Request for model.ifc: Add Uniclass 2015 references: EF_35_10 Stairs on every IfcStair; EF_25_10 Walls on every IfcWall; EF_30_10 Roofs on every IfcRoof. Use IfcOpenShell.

First a look at what the model holds.

```python
import ifcopenshell

model = ifcopenshell.open("model.ifc")
print(model.schema)
print("classifications:", [c.Name for c in model.by_type("IfcClassification")])
for ifc_class in ("IfcDoor", "IfcRoof", "IfcStair", "IfcWall", "IfcWindow"):
    print(ifc_class, len(model.by_type(ifc_class)))
```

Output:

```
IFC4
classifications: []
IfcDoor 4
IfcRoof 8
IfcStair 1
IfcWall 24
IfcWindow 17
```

```python
import ifcopenshell
import ifcopenshell.api.classification

model = ifcopenshell.open("model.ifc")

system = ifcopenshell.api.classification.add_classification(model, classification="Uniclass 2015")

codes = {
    "IfcStair": ("EF_35_10", "Stairs"),
    "IfcWall": ("EF_25_10", "Walls"),
    "IfcRoof": ("EF_30_10", "Roofs"),
}
for ifc_class, (code, name) in codes.items():
    products = model.by_type(ifc_class)
    ifcopenshell.api.classification.add_reference(
        model, products=products, classification=system, identification=code, name=name
    )
    print(code, len(products))

model.write("model_updated.ifc")
```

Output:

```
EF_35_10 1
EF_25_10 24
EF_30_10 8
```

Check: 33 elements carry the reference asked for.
